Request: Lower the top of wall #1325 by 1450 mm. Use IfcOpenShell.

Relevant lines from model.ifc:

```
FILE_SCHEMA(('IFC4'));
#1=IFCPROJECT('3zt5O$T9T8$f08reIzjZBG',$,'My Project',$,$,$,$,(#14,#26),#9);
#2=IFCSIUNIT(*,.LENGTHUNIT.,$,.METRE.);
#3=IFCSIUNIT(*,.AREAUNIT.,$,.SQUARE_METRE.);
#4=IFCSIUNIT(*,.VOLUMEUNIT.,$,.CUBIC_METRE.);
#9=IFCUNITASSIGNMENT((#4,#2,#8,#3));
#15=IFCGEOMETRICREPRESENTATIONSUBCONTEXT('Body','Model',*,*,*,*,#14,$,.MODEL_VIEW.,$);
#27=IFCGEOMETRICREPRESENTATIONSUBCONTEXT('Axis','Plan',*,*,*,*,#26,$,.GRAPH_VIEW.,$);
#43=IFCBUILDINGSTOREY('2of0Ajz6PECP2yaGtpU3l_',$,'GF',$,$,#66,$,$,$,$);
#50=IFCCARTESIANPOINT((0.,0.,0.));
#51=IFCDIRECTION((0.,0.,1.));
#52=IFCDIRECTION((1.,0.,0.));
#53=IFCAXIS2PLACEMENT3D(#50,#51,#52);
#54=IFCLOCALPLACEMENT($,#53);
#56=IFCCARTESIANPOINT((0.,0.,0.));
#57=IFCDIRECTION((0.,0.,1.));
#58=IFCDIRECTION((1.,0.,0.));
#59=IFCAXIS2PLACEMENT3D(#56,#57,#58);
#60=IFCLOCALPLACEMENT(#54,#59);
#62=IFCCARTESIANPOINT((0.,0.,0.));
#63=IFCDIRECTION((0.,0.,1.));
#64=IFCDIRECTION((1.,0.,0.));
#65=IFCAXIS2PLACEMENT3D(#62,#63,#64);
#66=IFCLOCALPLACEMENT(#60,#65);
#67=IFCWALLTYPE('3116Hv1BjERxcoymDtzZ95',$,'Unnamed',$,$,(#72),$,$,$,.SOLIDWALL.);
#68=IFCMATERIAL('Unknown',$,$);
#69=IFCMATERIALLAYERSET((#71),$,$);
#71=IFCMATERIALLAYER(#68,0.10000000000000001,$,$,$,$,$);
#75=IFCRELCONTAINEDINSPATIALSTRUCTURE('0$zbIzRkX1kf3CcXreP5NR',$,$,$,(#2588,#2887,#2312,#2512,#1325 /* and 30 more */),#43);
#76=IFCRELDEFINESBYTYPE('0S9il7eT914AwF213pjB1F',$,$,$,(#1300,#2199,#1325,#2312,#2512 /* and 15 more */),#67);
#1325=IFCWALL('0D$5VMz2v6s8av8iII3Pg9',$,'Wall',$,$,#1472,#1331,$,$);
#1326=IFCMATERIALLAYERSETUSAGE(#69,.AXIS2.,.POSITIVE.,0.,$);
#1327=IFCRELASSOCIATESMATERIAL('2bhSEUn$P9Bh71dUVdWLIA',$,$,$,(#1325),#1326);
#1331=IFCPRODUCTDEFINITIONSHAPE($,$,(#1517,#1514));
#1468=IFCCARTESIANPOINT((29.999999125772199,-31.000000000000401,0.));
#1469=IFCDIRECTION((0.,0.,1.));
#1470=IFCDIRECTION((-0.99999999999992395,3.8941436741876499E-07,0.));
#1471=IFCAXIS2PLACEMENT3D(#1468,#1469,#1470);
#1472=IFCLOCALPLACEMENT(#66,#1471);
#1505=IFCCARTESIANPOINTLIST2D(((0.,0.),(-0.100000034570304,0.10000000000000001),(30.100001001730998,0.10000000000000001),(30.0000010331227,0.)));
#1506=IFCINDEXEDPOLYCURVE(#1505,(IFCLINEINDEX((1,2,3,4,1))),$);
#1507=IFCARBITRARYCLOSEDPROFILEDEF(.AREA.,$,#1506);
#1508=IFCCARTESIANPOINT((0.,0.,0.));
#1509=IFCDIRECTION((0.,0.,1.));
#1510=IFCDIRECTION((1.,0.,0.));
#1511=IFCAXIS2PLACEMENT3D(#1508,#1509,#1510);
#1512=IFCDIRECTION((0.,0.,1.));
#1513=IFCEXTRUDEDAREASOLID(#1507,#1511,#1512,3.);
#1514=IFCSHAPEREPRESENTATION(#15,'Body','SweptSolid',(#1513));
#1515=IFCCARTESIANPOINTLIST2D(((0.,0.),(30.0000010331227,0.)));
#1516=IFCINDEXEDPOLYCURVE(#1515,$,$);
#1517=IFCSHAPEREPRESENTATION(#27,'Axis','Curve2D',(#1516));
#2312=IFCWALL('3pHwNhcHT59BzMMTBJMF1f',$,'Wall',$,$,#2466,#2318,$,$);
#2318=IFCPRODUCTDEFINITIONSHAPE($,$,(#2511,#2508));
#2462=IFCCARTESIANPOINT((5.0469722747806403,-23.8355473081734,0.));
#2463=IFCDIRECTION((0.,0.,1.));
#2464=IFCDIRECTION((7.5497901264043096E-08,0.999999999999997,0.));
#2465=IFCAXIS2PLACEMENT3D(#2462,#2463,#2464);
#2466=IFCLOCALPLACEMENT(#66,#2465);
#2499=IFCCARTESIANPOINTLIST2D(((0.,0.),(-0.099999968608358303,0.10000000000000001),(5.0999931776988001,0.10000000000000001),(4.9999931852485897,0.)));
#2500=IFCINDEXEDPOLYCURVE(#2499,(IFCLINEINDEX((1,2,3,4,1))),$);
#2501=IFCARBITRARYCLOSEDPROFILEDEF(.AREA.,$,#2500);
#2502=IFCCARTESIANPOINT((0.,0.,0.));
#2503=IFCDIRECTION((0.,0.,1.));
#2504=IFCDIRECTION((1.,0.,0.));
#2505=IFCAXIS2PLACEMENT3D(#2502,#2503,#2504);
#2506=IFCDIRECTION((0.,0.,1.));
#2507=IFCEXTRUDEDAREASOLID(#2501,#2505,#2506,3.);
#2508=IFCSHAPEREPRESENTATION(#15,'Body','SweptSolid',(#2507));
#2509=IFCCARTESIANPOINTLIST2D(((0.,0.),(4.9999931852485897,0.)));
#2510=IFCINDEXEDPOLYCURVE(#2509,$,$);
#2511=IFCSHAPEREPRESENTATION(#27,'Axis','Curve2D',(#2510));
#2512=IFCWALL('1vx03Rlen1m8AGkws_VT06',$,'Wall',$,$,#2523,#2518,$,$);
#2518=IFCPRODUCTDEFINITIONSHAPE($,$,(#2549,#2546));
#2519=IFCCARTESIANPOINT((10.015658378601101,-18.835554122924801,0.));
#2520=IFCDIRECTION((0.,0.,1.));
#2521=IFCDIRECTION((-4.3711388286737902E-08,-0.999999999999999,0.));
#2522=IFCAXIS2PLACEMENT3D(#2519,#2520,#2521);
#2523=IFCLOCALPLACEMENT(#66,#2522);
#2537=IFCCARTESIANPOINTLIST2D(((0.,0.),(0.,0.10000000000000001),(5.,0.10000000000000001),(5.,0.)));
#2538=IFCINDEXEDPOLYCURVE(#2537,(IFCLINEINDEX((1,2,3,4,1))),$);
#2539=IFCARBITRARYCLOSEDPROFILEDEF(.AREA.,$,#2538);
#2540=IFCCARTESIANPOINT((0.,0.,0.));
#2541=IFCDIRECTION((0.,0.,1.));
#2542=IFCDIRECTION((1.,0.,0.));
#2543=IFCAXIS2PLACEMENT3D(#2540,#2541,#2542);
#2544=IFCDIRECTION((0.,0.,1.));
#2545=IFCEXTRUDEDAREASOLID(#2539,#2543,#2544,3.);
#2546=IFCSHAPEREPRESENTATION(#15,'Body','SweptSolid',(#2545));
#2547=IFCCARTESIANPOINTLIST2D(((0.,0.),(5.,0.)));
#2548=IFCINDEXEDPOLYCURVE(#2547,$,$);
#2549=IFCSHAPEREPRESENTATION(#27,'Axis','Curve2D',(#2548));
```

```python
import ifcopenshell
import ifcopenshell.geom
import ifcopenshell.util.representation
import ifcopenshell.util.shape
import ifcopenshell.util.unit

model = ifcopenshell.open("model.ifc")
unit_scale = ifcopenshell.util.unit.calculate_unit_scale(model)
settings = ifcopenshell.geom.settings()


def volume(element):
    """Net volume in cubic metres, openings subtracted."""
    shape = ifcopenshell.geom.create_shape(settings, element)
    return ifcopenshell.util.shape.get_volume(shape.geometry)


wall = model.by_guid("0D$5VMz2v6s8av8iII3Pg9")
before = volume(wall)

body = ifcopenshell.util.representation.get_representation(wall, "Model", "Body")
solid = body.Items[0]
old_height = solid.Depth
solid.Depth -= 1.45 / unit_scale
after = volume(wall)

print(f"height {old_height:g} -> {solid.Depth:g}, volume {before:.3f} -> {after:.3f} m3")

model.write("model_v2.ifc")
```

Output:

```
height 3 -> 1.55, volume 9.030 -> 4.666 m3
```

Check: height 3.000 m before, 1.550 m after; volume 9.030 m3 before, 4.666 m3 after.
